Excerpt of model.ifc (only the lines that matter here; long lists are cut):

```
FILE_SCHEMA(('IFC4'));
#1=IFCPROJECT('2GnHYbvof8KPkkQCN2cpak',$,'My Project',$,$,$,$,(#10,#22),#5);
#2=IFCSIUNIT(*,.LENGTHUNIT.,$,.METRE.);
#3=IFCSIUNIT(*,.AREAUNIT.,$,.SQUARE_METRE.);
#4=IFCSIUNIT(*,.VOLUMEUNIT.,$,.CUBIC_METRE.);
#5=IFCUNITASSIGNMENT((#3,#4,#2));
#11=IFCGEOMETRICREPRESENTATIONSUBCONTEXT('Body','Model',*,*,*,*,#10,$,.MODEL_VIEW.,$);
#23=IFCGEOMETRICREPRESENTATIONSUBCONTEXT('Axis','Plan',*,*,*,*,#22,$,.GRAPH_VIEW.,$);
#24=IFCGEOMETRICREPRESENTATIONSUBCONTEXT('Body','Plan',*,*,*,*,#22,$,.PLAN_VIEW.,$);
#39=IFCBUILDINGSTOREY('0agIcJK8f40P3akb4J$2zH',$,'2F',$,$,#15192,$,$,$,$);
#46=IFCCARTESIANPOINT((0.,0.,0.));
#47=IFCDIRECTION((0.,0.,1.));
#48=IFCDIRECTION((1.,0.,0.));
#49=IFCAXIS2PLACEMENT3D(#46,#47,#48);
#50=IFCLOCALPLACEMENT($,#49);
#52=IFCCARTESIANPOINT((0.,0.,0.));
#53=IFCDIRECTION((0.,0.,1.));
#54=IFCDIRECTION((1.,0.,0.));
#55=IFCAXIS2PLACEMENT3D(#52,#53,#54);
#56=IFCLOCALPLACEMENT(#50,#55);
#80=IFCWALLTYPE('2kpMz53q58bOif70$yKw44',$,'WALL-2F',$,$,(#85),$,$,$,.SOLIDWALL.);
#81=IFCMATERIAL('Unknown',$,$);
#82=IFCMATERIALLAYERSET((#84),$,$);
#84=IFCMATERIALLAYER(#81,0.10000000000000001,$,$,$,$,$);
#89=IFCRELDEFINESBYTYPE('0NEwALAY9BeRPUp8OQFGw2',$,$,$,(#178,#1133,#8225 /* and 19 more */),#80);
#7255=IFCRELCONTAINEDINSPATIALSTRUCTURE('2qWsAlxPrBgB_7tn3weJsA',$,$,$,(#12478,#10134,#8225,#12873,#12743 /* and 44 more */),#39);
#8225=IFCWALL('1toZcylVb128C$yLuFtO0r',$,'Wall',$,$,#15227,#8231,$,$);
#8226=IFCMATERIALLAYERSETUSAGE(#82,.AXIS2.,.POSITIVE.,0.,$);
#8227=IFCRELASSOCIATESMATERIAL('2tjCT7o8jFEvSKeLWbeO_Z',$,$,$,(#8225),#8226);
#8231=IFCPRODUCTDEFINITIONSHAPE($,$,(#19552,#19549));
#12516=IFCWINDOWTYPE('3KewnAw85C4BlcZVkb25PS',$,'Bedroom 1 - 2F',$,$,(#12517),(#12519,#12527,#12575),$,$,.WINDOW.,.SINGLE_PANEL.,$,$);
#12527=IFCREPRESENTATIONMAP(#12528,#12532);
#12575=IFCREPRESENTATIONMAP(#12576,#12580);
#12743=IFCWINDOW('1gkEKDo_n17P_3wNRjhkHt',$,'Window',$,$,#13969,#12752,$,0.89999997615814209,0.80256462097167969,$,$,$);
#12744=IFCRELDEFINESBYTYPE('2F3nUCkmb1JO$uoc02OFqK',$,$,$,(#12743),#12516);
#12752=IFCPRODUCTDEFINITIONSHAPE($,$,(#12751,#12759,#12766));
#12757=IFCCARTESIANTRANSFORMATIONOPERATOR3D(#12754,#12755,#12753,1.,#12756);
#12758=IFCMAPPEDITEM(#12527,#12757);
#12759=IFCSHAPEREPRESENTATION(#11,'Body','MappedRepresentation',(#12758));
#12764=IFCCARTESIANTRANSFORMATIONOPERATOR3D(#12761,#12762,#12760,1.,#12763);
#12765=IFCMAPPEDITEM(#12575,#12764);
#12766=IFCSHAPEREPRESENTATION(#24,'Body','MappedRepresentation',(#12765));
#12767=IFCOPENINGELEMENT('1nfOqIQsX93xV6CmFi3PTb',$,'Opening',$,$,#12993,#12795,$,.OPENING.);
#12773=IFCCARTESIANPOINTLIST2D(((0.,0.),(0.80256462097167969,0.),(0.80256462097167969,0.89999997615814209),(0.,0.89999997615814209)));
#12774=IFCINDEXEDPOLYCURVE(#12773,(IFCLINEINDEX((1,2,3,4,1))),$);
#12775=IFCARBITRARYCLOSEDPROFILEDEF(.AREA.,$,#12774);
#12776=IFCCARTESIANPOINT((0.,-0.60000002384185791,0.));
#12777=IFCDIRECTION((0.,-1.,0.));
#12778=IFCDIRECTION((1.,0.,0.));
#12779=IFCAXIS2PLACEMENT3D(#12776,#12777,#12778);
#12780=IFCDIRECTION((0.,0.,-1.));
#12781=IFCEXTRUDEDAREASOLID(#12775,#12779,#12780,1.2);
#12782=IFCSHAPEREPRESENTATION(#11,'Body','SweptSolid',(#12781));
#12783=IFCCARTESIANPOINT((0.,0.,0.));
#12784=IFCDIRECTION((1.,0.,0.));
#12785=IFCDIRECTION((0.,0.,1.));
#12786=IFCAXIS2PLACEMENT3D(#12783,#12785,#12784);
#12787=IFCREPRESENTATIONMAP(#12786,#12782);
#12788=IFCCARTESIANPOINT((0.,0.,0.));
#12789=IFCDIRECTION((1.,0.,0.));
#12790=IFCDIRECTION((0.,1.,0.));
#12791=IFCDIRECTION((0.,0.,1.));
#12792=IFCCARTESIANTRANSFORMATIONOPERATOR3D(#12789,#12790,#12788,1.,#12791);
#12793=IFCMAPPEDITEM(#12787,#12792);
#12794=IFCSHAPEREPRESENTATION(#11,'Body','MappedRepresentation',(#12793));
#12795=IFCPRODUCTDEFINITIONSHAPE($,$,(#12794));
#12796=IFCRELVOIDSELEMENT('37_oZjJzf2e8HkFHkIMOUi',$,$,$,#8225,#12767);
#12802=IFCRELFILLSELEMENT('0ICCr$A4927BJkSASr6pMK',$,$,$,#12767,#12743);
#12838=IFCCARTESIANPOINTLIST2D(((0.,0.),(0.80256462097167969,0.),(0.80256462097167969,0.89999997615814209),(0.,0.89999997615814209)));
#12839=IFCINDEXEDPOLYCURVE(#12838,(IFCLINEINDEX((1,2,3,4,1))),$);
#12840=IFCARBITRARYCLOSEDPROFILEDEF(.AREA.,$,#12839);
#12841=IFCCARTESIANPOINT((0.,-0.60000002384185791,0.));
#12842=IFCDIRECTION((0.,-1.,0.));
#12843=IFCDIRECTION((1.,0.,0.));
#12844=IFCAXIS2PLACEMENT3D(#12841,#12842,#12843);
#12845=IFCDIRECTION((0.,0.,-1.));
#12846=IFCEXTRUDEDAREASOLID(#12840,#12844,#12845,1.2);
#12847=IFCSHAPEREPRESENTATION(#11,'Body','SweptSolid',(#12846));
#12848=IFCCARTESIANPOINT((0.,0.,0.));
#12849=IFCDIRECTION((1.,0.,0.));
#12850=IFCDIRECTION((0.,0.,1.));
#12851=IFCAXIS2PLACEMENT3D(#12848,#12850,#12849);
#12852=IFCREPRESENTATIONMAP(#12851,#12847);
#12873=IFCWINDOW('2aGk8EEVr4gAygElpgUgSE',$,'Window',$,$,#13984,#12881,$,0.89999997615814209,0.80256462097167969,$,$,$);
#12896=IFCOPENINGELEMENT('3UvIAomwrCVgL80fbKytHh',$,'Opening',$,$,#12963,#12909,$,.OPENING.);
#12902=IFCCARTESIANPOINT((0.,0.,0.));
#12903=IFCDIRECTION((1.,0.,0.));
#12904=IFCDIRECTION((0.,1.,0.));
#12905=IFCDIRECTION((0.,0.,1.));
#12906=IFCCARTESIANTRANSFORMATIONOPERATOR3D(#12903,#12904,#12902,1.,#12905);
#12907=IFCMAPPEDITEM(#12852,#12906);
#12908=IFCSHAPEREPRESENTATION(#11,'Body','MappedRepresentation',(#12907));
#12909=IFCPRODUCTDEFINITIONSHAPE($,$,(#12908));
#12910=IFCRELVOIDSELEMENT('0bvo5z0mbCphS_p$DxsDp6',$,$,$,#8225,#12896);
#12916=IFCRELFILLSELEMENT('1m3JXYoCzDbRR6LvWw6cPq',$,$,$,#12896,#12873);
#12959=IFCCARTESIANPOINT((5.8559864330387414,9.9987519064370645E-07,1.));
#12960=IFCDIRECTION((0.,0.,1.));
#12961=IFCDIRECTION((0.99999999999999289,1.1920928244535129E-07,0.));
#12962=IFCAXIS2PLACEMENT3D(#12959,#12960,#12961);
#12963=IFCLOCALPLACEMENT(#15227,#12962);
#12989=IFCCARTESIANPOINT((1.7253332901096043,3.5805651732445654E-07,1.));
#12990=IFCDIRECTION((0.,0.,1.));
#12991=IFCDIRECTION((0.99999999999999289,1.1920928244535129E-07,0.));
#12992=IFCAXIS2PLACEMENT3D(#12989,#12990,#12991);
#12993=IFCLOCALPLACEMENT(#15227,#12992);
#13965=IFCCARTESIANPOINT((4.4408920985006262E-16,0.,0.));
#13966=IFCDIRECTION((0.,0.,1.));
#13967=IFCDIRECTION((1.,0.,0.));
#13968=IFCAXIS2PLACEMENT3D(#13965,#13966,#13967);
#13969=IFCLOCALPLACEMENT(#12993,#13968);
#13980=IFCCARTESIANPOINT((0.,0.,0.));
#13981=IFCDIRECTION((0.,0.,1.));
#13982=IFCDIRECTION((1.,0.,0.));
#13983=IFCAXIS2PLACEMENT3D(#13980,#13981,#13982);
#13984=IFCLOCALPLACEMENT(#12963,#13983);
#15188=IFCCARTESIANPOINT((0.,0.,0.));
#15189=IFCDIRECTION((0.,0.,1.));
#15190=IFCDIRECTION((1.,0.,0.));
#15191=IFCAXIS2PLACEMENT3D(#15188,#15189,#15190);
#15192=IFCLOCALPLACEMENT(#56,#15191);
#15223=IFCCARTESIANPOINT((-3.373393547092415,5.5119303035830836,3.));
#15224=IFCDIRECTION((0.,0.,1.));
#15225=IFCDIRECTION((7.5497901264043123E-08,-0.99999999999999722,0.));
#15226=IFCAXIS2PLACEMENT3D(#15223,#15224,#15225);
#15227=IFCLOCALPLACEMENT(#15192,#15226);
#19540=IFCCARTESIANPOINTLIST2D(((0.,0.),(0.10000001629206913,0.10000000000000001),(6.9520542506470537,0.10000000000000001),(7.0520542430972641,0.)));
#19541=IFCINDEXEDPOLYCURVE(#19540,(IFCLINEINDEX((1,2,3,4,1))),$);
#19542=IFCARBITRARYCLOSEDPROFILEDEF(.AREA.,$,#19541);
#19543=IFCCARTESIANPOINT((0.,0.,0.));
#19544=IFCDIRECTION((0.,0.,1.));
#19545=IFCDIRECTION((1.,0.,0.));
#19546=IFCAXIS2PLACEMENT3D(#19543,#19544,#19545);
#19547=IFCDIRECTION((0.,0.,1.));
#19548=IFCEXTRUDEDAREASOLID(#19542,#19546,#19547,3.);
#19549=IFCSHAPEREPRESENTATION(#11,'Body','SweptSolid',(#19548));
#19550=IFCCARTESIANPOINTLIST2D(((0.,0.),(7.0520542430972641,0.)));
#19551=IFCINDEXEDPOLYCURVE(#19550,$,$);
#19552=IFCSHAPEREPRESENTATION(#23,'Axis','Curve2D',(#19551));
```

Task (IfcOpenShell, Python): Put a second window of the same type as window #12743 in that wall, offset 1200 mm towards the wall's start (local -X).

```python
import ifcopenshell
import ifcopenshell.api.feature
import ifcopenshell.api.geometry
import ifcopenshell.api.root
import ifcopenshell.geom
import ifcopenshell.util.element
import ifcopenshell.util.placement
import ifcopenshell.util.shape
import ifcopenshell.util.unit

model = ifcopenshell.open("model.ifc")
unit_scale = ifcopenshell.util.unit.calculate_unit_scale(model)
settings = ifcopenshell.geom.settings()


def volume(element):
    """Net volume in cubic metres, openings subtracted."""
    shape = ifcopenshell.geom.create_shape(settings, element)
    return ifcopenshell.util.shape.get_volume(shape.geometry)


window = model.by_id(12743)
opening = window.FillsVoids[0].RelatingOpeningElement
wall = opening.VoidsElements[0].RelatingBuildingElement
before = volume(wall)
shift = ifcopenshell.util.placement.get_local_placement(wall.ObjectPlacement)[:3, 0] * -1.2 / unit_scale

# copy_class copies the void relationship, type, container and properties, but no geometry.
new_opening = ifcopenshell.api.root.copy_class(model, product=opening)
new_opening.Representation = ifcopenshell.util.element.copy_deep(
    model, opening.Representation, exclude=["IfcGeometricRepresentationContext", "IfcRepresentationMap"]
)
new_window = ifcopenshell.api.root.copy_class(model, product=window)
new_window.Representation = ifcopenshell.util.element.copy_deep(
    model, window.Representation, exclude=["IfcGeometricRepresentationContext", "IfcRepresentationMap"]
)
ifcopenshell.api.feature.add_filling(model, opening=new_opening, element=new_window)

for old, new in ((opening, new_opening), (window, new_window)):
    matrix = ifcopenshell.util.placement.get_local_placement(old.ObjectPlacement)
    matrix[:3, 3] += shift
    ifcopenshell.api.geometry.edit_object_placement(model, product=new, matrix=matrix, is_si=False)

after = volume(wall)

print(f"wall volume {before:.3f} -> {after:.3f} m3")

model.write("model_rev.ifc")
```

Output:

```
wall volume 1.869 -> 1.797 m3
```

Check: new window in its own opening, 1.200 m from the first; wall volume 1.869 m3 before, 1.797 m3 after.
